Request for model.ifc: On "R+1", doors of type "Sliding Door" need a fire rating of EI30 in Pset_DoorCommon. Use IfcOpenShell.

First a look at what the model holds.

```python
import ifcopenshell
import ifcopenshell.util.element

model = ifcopenshell.open("model.ifc")
print(model.schema)
storey = next(s for s in model.by_type("IfcBuildingStorey") if s.Name == "R+1")
doors = [e for e in ifcopenshell.util.element.get_decomposition(storey) if e.is_a("IfcDoor")]
seen = {}
for e in doors:
    element_type = ifcopenshell.util.element.get_type(e)
    key = (element_type.Name if element_type != e and element_type else None, ifcopenshell.util.element.get_pset(e, "Pset_DoorCommon", "FireRating"))
    seen[key] = seen.get(key, 0) + 1
for (name, value), count in sorted(seen.items(), key=str):
    print(count, "x", name, "|", value)
```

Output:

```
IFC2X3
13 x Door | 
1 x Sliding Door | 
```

```python
import ifcopenshell
import ifcopenshell.api.pset
import ifcopenshell.util.element

model = ifcopenshell.open("model.ifc")

storey = next(s for s in model.by_type("IfcBuildingStorey") if s.Name == "R+1")
doors = [e for e in ifcopenshell.util.element.get_decomposition(storey) if e.is_a("IfcDoor")]

count = 0
for e in doors:
    element_type = ifcopenshell.util.element.get_type(e)
    if element_type in (None, e) or element_type.Name != "Sliding Door":
        continue
    # add_pset returns the element's existing set when there is one.
    pset = ifcopenshell.api.pset.add_pset(model, product=e, name="Pset_DoorCommon")
    ifcopenshell.api.pset.edit_pset(model, pset=pset, properties={"FireRating": "EI30"})
    count += 1

print(count, "doors updated")

model.write("model_edited.ifc")
```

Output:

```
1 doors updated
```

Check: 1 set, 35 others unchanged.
